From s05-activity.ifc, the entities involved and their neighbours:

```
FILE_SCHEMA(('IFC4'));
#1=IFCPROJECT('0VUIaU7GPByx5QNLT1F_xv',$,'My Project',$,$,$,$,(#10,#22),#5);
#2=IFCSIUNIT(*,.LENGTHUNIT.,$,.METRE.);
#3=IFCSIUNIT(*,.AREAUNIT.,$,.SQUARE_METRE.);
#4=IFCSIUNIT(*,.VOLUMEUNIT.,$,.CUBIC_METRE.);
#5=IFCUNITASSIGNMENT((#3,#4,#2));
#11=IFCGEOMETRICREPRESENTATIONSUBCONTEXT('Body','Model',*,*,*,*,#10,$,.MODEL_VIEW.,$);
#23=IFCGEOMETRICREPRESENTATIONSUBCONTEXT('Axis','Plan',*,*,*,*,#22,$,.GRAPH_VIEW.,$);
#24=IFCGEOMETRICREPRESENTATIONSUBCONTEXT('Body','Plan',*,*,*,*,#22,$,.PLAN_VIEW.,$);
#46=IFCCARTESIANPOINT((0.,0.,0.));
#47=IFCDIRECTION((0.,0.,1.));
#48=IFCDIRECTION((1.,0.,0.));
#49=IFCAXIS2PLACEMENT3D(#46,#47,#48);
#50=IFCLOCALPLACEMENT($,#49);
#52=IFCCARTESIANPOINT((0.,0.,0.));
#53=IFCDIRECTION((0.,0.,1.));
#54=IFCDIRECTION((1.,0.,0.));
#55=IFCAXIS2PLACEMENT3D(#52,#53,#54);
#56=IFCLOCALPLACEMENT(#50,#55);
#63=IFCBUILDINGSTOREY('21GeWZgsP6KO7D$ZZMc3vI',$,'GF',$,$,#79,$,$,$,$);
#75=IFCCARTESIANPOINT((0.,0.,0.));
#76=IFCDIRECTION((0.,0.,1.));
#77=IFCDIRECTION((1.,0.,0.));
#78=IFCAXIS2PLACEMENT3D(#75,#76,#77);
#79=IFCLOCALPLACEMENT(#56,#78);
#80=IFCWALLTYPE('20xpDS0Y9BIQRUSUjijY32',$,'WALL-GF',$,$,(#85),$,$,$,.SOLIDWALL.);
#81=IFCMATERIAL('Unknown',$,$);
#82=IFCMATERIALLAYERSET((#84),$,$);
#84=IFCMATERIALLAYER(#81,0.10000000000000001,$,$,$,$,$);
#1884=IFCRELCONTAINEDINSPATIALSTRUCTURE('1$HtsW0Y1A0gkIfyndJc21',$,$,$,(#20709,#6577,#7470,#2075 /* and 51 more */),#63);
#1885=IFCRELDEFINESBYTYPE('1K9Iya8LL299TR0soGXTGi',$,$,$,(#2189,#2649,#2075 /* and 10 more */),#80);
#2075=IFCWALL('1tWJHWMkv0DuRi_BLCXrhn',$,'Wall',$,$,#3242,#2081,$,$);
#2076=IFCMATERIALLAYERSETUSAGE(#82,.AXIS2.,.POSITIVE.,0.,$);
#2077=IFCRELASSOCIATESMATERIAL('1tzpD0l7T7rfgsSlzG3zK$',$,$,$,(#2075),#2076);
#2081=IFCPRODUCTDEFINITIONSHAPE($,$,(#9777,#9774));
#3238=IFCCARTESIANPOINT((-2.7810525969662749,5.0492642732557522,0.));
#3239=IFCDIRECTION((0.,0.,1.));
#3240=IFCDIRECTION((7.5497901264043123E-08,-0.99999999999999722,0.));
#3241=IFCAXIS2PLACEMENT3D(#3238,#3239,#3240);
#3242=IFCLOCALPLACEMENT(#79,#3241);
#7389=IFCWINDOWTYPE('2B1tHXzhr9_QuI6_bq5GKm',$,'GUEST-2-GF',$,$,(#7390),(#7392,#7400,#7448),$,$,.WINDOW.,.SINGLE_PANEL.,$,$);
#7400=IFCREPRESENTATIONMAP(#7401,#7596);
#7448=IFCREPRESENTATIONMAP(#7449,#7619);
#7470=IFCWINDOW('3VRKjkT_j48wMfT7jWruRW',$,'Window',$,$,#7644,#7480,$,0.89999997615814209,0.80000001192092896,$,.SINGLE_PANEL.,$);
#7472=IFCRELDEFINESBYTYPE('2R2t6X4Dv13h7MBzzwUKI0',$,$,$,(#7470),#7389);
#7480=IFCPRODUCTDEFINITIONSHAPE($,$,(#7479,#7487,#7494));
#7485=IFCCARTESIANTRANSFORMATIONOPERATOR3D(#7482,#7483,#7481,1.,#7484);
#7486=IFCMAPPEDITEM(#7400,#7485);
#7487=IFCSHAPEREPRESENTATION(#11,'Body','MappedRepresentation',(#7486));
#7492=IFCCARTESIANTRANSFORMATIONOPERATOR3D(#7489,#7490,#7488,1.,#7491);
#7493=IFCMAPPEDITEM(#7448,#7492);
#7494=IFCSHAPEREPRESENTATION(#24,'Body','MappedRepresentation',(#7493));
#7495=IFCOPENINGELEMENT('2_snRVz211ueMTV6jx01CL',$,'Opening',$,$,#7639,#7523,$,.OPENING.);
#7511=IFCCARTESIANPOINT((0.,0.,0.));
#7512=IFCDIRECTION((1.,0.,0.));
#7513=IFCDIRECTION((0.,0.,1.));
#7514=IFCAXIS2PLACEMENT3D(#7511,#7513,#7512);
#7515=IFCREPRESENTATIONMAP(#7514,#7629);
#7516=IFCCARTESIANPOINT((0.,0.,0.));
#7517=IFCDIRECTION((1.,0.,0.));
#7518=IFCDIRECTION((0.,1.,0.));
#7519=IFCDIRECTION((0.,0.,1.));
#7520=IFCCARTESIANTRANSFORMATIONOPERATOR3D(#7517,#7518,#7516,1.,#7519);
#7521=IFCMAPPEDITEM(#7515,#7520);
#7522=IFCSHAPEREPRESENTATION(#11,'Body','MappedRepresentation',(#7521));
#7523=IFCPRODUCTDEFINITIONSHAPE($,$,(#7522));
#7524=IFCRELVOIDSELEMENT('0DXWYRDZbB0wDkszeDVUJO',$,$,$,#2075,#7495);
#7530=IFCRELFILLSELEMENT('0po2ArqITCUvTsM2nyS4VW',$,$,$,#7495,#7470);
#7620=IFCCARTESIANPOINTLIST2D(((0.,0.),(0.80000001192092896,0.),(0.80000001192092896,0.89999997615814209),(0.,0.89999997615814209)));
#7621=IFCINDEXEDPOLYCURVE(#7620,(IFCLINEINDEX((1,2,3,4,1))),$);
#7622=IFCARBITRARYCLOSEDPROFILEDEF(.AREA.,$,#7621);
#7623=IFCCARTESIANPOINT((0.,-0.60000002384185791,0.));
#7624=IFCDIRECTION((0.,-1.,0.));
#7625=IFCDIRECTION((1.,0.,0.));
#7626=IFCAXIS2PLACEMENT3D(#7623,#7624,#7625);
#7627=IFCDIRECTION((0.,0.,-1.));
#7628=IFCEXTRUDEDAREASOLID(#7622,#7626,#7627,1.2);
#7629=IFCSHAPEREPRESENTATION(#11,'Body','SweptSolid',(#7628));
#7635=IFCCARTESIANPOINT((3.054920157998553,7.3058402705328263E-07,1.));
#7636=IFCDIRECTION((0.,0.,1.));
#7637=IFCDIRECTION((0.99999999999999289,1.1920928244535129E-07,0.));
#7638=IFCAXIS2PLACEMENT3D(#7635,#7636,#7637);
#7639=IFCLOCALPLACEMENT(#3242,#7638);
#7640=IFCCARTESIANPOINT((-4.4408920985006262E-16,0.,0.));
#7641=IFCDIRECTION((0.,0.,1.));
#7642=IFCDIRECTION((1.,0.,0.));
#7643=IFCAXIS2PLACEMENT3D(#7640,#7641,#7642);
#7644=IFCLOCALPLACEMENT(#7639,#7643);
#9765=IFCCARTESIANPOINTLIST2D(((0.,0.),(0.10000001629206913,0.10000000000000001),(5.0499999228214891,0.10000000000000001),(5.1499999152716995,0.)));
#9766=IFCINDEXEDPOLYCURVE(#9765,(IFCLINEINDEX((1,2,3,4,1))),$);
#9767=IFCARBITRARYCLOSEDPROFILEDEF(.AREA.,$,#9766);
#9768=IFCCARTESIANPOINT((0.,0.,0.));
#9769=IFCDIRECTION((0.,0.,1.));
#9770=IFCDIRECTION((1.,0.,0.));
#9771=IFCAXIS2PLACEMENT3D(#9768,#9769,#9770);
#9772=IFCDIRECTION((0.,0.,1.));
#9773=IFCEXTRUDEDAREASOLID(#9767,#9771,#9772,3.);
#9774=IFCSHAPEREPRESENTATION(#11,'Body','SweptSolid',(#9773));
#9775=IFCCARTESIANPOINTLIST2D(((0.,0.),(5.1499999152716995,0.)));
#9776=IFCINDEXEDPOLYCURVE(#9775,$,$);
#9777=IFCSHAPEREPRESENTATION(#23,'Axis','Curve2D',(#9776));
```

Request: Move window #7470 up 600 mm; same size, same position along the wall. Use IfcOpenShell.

```python
import numpy as np
import ifcopenshell
import ifcopenshell.api.geometry
import ifcopenshell.util.placement
import ifcopenshell.util.unit

model = ifcopenshell.open("s05-activity.ifc")
unit_scale = ifcopenshell.util.unit.calculate_unit_scale(model)

window = model.by_guid("3VRKjkT_j48wMfT7jWruRW")
opening = window.FillsVoids[0].RelatingOpeningElement
dz = 0.6

shift = np.array([0.0, 0.0, dz])
# The window is placed relative to its opening, so it follows when the opening moves.
matrix = ifcopenshell.util.placement.get_local_placement(opening.ObjectPlacement)
matrix[:3, 3] += shift
ifcopenshell.api.geometry.edit_object_placement(
    model, product=opening, matrix=matrix, is_si=False, should_transform_children=True
)

print(f"moved by {dz * unit_scale:+.3f} m")

model.write("s05-activity-out.ifc")
```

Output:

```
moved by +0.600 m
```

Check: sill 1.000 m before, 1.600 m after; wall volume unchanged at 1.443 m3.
